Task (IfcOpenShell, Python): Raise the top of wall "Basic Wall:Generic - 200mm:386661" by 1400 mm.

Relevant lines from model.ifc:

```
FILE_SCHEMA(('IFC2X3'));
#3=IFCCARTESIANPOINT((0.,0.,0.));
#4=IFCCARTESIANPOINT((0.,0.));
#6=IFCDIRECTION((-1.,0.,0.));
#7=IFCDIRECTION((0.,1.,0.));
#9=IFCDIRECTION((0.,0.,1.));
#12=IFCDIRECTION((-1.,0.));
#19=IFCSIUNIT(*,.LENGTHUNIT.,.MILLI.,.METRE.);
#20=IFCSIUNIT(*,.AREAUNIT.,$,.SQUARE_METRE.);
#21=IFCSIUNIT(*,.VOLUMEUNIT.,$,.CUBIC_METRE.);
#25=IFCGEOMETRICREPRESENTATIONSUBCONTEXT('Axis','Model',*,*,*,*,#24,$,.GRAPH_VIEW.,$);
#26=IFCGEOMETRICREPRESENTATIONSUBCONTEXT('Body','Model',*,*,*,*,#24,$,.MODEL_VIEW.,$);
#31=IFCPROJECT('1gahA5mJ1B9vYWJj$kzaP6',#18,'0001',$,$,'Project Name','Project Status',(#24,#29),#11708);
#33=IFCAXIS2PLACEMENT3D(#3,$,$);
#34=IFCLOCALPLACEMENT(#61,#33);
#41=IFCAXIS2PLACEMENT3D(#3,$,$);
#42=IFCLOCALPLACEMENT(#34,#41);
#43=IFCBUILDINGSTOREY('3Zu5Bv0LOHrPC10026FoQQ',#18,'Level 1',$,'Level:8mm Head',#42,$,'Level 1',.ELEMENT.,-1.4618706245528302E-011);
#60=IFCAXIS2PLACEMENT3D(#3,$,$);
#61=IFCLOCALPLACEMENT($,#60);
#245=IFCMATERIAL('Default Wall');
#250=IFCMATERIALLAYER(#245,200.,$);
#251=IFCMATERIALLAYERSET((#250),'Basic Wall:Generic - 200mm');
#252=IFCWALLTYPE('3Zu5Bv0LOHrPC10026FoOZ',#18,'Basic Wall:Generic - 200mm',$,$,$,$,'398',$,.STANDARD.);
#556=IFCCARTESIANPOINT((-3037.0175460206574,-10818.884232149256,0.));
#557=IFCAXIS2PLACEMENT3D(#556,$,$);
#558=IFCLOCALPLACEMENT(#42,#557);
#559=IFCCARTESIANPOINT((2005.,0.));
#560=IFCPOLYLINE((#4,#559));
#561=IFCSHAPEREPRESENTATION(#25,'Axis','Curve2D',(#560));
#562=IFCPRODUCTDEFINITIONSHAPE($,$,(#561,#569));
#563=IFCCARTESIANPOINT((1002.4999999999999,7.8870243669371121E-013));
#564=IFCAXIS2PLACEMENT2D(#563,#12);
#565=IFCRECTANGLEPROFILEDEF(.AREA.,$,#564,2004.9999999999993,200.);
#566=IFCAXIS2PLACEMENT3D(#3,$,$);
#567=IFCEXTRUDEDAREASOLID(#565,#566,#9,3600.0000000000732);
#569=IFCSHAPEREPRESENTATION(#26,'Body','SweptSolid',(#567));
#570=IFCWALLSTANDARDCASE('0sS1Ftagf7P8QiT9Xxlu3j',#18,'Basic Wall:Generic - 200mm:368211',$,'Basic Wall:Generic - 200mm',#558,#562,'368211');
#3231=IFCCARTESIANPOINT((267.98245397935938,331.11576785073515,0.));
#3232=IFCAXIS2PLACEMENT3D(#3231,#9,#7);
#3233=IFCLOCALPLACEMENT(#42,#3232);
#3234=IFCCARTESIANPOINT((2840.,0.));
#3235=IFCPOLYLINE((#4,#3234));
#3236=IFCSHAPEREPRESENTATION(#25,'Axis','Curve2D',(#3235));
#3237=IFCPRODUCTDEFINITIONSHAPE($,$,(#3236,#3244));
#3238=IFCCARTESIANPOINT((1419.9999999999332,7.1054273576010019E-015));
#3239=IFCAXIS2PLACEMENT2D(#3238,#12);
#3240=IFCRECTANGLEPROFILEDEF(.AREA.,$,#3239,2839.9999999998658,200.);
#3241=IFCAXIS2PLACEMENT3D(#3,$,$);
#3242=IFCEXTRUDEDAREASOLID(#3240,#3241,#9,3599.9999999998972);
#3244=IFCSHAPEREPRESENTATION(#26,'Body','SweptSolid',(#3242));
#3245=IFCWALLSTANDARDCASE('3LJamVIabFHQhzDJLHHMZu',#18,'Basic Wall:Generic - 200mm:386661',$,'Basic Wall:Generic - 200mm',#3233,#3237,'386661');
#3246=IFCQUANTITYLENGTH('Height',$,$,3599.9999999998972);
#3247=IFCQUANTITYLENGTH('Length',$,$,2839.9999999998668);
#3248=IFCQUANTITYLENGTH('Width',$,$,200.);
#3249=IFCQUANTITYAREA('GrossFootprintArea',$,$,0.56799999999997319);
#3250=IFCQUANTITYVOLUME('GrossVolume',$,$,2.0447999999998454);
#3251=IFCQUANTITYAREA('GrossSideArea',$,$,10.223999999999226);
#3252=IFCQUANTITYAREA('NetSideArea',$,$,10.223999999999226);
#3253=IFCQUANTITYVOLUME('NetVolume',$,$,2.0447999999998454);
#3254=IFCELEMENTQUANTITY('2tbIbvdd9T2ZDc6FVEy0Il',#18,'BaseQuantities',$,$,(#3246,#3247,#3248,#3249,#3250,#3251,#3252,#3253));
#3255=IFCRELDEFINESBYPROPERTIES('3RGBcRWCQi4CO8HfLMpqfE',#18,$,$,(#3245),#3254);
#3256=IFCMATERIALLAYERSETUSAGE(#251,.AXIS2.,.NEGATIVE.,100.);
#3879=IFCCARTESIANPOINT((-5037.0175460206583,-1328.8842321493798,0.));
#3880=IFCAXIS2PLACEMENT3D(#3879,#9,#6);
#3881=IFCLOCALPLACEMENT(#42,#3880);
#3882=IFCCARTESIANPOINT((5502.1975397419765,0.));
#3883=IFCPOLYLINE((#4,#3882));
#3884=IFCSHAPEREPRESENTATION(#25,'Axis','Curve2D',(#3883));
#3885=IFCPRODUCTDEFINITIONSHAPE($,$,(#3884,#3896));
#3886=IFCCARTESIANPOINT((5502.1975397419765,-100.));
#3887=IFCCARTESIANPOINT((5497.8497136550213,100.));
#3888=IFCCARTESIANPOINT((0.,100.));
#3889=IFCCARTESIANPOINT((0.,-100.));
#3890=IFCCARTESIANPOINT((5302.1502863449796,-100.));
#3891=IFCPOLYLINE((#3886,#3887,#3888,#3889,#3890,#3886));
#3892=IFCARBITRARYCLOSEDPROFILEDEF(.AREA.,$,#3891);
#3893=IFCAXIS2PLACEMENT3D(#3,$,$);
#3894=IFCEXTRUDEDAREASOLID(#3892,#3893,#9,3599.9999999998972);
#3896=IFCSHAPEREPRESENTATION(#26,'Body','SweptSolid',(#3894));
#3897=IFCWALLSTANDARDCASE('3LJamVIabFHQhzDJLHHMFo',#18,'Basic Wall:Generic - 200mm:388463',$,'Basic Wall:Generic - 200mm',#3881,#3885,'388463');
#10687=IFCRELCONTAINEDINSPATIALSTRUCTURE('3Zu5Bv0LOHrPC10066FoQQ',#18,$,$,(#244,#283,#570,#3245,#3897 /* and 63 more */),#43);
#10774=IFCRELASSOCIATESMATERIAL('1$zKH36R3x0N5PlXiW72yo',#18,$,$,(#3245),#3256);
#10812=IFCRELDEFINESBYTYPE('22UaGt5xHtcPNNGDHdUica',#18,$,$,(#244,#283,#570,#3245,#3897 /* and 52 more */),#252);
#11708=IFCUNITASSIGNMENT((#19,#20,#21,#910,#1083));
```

```python
import ifcopenshell
import ifcopenshell.api.pset
import ifcopenshell.geom
import ifcopenshell.util.element
import ifcopenshell.util.representation
import ifcopenshell.util.shape
import ifcopenshell.util.unit

model = ifcopenshell.open("model.ifc")
unit_scale = ifcopenshell.util.unit.calculate_unit_scale(model)
area_scale = ifcopenshell.util.unit.calculate_unit_scale(model, "AREAUNIT")
volume_scale = ifcopenshell.util.unit.calculate_unit_scale(model, "VOLUMEUNIT")
settings = ifcopenshell.geom.settings()


def volume(element):
    """Net volume in cubic metres, openings subtracted."""
    shape = ifcopenshell.geom.create_shape(settings, element)
    return ifcopenshell.util.shape.get_volume(shape.geometry)


wall = model.by_guid("3LJamVIabFHQhzDJLHHMZu")
before = volume(wall)

body = ifcopenshell.util.representation.get_representation(wall, "Model", "Body")
solid = body.Items[0]
old_height = solid.Depth
solid.Depth += 1.4 / unit_scale
after = volume(wall)
thickness = 0.2  # wall thickness in metres

# Update the stored height, areas and volumes.
qto = model.by_id(ifcopenshell.util.element.get_pset(wall, "BaseQuantities", should_inherit=False)["id"])
ifcopenshell.api.pset.edit_qto(model, qto=qto, properties={
    "Height": solid.Depth,
    "GrossVolume": ifcopenshell.util.element.get_pset(wall, "BaseQuantities", "GrossVolume") * solid.Depth / old_height,
    "GrossSideArea": ifcopenshell.util.element.get_pset(wall, "BaseQuantities", "GrossSideArea") * solid.Depth / old_height,
    "NetSideArea": after / thickness / area_scale,
    "NetVolume": after / volume_scale,
})

print(f"height {old_height:g} -> {solid.Depth:g}, volume {before:.3f} -> {after:.3f} m3")

model.write("model-out.ifc")
```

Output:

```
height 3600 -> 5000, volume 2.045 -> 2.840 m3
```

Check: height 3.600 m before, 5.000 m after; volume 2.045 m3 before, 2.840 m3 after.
